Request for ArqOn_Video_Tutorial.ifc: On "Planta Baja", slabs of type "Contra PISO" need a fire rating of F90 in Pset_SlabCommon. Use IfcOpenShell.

First a look at what the model holds.

```python
import ifcopenshell
import ifcopenshell.util.element

model = ifcopenshell.open("ArqOn_Video_Tutorial.ifc")
print(model.schema)
storey = next(s for s in model.by_type("IfcBuildingStorey") if s.Name == "Planta Baja")
slabs = [e for e in ifcopenshell.util.element.get_decomposition(storey) if e.is_a("IfcSlab")]
seen = {}
for e in slabs:
    element_type = ifcopenshell.util.element.get_type(e)
    key = (element_type.Name if element_type != e and element_type else None, ifcopenshell.util.element.get_pset(e, "Pset_SlabCommon", "FireRating"))
    seen[key] = seen.get(key, 0) + 1
for (name, value), count in sorted(seen.items(), key=str):
    print(count, "x", name, "|", value)
```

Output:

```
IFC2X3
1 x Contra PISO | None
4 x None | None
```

```python
import ifcopenshell
import ifcopenshell.api.pset
import ifcopenshell.util.element

model = ifcopenshell.open("ArqOn_Video_Tutorial.ifc")

storey = next(s for s in model.by_type("IfcBuildingStorey") if s.Name == "Planta Baja")
slabs = [e for e in ifcopenshell.util.element.get_decomposition(storey) if e.is_a("IfcSlab")]

count = 0
for e in slabs:
    element_type = ifcopenshell.util.element.get_type(e)
    if element_type in (None, e) or element_type.Name != "Contra PISO":
        continue
    # add_pset returns the element's existing set when there is one.
    pset = ifcopenshell.api.pset.add_pset(model, product=e, name="Pset_SlabCommon")
    ifcopenshell.api.pset.edit_pset(model, pset=pset, properties={"FireRating": "F90"})
    count += 1

print(count, "slabs updated")

model.write("ArqOn_Video_Tutorial_edited.ifc")
```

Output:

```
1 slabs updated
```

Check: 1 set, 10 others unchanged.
